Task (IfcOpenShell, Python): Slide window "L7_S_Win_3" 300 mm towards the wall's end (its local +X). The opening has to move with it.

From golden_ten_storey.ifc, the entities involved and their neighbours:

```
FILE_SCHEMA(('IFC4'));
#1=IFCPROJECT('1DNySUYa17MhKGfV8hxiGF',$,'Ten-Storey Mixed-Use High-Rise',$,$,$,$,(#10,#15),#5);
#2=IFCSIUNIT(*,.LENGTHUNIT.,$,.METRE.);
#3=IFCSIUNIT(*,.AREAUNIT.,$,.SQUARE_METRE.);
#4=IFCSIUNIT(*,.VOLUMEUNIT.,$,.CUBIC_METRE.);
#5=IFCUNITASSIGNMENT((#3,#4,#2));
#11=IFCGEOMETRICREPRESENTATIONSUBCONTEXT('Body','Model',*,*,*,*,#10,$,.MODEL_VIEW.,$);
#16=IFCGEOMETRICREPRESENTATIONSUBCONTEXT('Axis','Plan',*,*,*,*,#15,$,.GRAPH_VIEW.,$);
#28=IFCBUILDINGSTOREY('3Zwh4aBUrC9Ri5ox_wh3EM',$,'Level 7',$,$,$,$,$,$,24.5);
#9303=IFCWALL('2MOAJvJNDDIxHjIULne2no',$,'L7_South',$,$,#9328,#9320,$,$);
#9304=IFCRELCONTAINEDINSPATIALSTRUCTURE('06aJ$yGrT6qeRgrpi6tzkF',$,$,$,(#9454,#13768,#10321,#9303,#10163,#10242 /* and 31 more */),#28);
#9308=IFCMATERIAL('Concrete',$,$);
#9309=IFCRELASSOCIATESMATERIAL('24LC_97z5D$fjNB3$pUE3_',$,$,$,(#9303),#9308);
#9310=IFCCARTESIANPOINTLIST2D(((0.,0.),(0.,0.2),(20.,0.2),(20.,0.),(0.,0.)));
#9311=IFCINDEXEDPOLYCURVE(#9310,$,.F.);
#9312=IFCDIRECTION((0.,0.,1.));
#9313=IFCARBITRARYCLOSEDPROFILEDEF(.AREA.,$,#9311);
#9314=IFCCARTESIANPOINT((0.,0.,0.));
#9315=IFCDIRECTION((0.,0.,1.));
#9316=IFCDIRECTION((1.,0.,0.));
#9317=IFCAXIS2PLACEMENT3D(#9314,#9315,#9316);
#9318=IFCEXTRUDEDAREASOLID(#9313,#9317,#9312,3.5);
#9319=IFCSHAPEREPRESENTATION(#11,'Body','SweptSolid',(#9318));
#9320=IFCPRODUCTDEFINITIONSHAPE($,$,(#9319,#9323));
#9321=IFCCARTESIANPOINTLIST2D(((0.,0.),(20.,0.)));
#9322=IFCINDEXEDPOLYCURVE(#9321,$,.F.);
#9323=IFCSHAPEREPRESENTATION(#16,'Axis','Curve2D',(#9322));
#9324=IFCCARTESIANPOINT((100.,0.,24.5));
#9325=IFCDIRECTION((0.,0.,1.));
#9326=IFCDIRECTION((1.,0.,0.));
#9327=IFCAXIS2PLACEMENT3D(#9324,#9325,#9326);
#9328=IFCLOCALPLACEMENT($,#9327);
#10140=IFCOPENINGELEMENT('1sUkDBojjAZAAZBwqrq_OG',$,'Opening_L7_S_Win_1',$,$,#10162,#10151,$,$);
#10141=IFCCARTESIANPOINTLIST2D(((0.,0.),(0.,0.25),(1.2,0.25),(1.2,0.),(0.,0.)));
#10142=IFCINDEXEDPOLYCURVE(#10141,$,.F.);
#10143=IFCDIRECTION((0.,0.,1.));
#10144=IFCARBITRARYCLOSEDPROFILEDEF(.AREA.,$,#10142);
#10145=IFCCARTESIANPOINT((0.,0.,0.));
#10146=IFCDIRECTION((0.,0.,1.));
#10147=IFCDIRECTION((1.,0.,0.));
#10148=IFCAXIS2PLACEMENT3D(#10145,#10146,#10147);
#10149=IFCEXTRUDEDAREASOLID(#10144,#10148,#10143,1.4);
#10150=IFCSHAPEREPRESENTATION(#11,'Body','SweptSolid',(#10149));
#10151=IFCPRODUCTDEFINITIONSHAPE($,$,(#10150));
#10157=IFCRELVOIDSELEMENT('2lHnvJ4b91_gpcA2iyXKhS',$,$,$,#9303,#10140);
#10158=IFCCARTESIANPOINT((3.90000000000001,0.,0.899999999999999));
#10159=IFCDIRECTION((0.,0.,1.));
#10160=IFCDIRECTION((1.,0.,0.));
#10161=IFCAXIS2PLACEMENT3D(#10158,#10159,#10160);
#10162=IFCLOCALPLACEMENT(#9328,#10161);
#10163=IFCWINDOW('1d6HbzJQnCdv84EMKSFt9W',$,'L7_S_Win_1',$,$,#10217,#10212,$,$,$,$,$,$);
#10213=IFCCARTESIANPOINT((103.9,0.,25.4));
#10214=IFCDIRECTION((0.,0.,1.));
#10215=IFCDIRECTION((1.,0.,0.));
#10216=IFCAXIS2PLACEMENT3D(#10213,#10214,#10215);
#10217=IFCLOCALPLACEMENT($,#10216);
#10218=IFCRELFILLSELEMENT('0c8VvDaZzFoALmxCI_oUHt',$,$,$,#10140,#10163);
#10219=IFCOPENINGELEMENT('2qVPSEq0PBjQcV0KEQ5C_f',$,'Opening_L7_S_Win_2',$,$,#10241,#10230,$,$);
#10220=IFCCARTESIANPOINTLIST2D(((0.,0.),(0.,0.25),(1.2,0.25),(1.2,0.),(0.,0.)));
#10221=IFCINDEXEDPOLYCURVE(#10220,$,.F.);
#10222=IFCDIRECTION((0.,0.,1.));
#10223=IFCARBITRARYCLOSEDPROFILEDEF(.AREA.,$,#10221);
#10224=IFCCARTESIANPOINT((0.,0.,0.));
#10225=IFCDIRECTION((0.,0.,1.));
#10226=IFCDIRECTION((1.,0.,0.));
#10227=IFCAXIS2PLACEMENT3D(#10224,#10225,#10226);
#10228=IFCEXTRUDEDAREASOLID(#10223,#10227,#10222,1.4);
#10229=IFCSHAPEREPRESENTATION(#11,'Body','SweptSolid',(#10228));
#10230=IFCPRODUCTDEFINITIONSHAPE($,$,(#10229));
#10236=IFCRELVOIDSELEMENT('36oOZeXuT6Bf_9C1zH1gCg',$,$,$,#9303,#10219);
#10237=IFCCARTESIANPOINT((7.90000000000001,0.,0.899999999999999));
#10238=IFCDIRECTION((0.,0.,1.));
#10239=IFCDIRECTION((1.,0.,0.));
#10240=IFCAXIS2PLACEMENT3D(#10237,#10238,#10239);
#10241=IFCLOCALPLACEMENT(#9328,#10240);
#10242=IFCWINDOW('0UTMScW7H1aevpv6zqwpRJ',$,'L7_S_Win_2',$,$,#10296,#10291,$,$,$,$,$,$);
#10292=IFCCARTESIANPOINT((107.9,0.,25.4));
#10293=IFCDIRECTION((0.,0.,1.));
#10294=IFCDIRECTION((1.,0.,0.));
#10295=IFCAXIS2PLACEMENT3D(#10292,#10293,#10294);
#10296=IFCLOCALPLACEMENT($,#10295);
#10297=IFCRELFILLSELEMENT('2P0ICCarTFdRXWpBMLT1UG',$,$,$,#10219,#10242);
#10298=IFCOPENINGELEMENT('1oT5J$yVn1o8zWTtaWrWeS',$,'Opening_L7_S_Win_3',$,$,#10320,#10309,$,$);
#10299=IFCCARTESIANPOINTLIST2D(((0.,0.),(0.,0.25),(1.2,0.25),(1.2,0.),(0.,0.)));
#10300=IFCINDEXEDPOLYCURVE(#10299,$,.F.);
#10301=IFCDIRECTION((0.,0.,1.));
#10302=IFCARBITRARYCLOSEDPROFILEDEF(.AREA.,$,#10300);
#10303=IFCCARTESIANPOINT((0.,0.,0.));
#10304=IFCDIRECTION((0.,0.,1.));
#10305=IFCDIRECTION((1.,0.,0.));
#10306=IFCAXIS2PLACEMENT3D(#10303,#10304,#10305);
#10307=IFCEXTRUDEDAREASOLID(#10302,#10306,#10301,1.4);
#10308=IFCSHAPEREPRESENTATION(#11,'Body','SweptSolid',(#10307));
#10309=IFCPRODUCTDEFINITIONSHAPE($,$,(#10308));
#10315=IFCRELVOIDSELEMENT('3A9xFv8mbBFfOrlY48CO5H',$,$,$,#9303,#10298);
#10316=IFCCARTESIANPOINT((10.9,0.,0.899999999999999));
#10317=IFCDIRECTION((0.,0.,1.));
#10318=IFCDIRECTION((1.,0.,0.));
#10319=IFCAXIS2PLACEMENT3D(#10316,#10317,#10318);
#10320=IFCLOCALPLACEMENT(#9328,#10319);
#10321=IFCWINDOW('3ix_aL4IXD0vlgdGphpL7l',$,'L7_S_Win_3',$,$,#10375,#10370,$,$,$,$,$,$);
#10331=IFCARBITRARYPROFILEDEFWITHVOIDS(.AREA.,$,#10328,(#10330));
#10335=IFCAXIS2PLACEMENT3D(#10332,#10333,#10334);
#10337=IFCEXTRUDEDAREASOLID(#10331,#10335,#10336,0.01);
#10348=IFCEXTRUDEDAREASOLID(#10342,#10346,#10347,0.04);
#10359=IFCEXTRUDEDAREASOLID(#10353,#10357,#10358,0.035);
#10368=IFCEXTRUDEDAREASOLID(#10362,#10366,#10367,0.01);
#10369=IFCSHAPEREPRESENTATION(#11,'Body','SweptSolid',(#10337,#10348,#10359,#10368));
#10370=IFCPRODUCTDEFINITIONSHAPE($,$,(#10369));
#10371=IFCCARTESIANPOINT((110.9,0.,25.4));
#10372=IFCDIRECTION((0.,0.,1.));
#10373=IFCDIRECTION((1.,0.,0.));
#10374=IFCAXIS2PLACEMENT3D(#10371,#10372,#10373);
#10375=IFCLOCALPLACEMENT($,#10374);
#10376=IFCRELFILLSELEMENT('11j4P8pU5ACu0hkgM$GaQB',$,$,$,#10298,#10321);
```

```python
import ifcopenshell
import ifcopenshell.api.geometry
import ifcopenshell.util.placement
import ifcopenshell.util.unit

model = ifcopenshell.open("golden_ten_storey.ifc")
unit_scale = ifcopenshell.util.unit.calculate_unit_scale(model)

window = model.by_id(10321)
opening = window.FillsVoids[0].RelatingOpeningElement
wall = opening.VoidsElements[0].RelatingBuildingElement

wall_matrix = ifcopenshell.util.placement.get_local_placement(wall.ObjectPlacement)
shift = wall_matrix[:3, 0] * 0.3 / unit_scale
before = ifcopenshell.util.placement.get_local_placement(window.ObjectPlacement)[:3, 3].copy()

# The window is not placed relative to its opening, so move both.
for product in (opening, window):
    matrix = ifcopenshell.util.placement.get_local_placement(product.ObjectPlacement)
    matrix[:3, 3] += shift
    ifcopenshell.api.geometry.edit_object_placement(model, product=product, matrix=matrix, is_si=False)

after = ifcopenshell.util.placement.get_local_placement(window.ObjectPlacement)[:3, 3]
print("window moved by", (after - before).round(3) + 0.0)

model.write("golden_ten_storey-out.ifc")
```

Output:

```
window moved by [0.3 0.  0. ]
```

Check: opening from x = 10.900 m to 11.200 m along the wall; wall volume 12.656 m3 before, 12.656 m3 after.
